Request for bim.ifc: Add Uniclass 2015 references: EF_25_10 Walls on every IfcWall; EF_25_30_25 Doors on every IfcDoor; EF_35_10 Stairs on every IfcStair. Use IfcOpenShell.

First a look at what the model holds.

```python
import ifcopenshell

model = ifcopenshell.open("bim.ifc")
print(model.schema)
print("classifications:", [c.Name for c in model.by_type("IfcClassification")])
for ifc_class in ("IfcDoor", "IfcRoof", "IfcStair", "IfcWall", "IfcWindow"):
    print(ifc_class, len(model.by_type(ifc_class)))
```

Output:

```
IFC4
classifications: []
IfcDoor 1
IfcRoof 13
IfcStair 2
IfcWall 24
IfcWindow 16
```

```python
import ifcopenshell
import ifcopenshell.api.classification

model = ifcopenshell.open("bim.ifc")

system = ifcopenshell.api.classification.add_classification(model, classification="Uniclass 2015")

codes = {
    "IfcWall": ("EF_25_10", "Walls"),
    "IfcDoor": ("EF_25_30_25", "Doors"),
    "IfcStair": ("EF_35_10", "Stairs"),
}
for ifc_class, (code, name) in codes.items():
    products = model.by_type(ifc_class)
    ifcopenshell.api.classification.add_reference(
        model, products=products, classification=system, identification=code, name=name
    )
    print(code, len(products))

model.write("bim-out.ifc")
```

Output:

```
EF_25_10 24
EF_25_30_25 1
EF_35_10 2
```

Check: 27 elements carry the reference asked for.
